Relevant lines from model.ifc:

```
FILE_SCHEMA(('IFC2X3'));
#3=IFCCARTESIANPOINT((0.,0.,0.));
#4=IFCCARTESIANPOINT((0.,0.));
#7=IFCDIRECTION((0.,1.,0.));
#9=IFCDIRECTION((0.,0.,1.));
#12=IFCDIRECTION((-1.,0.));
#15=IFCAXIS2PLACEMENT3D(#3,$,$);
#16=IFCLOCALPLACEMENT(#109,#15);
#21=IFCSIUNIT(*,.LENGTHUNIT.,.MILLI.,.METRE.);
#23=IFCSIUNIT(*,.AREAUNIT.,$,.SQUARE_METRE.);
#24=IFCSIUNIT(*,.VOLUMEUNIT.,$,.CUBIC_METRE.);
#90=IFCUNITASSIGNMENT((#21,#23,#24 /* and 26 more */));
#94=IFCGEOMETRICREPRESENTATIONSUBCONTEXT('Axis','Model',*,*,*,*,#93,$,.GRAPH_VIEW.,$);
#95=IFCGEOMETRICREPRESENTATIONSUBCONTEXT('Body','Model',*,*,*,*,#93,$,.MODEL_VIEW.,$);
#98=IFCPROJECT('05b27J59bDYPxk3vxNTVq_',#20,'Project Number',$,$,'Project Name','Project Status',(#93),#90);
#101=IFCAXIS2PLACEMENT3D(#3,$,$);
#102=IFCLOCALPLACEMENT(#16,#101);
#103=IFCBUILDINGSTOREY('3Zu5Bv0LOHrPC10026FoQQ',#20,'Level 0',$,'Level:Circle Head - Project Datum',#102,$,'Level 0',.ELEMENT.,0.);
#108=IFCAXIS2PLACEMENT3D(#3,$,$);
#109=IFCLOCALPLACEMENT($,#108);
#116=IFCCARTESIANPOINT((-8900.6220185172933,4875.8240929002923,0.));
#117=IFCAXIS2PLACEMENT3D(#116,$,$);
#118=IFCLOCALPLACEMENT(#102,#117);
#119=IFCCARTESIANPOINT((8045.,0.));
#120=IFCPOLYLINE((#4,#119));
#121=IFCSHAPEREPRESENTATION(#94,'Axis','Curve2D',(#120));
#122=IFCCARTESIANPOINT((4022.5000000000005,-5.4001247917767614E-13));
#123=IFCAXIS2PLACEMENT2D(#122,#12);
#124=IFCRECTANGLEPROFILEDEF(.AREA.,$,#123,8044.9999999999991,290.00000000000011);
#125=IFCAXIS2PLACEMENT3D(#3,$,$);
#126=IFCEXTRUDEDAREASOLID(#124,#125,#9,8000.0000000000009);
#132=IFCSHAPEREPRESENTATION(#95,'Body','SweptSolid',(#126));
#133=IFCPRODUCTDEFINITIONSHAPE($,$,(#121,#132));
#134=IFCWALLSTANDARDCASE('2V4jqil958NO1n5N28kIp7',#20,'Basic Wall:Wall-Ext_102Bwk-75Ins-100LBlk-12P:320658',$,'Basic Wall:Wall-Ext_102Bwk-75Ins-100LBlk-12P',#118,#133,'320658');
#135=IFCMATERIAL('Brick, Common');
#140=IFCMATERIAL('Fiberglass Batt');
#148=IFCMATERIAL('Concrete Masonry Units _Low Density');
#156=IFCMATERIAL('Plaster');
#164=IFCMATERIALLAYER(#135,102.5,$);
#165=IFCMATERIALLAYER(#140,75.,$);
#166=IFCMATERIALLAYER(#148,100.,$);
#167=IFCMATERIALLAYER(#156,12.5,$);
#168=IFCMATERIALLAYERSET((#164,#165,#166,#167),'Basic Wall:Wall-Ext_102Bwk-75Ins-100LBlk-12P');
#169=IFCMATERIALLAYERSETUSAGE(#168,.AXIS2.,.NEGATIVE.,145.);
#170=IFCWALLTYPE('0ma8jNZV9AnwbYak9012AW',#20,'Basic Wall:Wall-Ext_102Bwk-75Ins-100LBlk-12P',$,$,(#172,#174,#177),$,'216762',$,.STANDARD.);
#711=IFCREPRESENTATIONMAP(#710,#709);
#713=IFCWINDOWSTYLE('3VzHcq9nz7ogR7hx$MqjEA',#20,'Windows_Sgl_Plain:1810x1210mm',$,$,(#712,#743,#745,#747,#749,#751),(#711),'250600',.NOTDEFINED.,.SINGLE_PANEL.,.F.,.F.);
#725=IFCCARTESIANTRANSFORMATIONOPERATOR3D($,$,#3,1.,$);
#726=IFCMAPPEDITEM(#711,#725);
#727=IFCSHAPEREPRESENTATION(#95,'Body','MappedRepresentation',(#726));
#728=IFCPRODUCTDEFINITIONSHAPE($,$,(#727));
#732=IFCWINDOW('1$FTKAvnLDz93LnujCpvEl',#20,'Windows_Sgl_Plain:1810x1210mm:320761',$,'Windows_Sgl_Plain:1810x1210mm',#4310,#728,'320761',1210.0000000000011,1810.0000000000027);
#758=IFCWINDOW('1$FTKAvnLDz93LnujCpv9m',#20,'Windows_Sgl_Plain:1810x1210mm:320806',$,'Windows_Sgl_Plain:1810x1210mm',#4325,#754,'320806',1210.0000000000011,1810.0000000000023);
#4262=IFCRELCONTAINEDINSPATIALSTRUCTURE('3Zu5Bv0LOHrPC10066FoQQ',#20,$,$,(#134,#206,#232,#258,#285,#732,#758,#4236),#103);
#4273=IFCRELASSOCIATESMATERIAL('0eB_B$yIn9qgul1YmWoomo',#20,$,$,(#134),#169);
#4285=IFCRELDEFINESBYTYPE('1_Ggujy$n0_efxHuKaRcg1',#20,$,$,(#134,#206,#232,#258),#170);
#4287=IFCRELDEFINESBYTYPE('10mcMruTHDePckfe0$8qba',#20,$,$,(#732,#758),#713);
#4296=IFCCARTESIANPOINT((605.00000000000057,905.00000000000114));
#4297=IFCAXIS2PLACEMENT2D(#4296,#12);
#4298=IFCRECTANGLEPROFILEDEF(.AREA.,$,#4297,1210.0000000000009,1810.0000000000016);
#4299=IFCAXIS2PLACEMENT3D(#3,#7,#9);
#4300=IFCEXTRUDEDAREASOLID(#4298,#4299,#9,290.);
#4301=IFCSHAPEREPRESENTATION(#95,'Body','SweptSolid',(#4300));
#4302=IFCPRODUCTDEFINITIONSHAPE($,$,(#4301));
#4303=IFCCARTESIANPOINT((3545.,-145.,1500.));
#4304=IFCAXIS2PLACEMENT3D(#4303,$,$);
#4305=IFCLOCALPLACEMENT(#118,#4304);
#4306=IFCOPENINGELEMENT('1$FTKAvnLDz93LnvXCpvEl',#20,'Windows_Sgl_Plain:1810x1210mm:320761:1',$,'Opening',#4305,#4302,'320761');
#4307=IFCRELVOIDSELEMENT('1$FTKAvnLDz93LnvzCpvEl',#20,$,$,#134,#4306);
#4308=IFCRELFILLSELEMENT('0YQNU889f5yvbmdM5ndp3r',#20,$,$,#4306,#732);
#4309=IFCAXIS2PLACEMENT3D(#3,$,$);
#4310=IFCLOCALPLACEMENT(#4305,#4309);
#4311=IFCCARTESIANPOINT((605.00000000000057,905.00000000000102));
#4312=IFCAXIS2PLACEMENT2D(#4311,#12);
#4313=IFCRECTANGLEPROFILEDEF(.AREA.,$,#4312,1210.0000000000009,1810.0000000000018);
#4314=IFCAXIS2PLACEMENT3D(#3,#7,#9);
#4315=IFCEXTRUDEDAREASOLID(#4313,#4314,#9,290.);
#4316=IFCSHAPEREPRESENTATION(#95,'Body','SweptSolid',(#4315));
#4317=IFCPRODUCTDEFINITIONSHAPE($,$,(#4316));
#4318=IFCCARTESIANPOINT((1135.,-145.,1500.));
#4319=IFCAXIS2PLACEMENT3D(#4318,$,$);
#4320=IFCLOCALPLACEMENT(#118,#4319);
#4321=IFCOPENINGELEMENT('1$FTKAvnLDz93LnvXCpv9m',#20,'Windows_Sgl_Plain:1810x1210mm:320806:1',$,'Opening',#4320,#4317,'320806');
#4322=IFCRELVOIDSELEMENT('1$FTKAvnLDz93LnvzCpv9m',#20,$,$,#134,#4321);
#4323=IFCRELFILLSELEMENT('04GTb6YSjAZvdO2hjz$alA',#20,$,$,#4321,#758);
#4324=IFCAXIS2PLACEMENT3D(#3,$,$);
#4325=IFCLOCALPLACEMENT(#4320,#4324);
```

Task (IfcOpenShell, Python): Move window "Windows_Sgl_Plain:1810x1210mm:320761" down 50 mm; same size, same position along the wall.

```python
import numpy as np
import ifcopenshell
import ifcopenshell.api.geometry
import ifcopenshell.util.placement
import ifcopenshell.util.unit

model = ifcopenshell.open("model.ifc")
unit_scale = ifcopenshell.util.unit.calculate_unit_scale(model)

window = model.by_guid("1$FTKAvnLDz93LnujCpvEl")
opening = window.FillsVoids[0].RelatingOpeningElement
dz = -50.0

shift = np.array([0.0, 0.0, dz])
# The window is placed relative to its opening, so it follows when the opening moves.
matrix = ifcopenshell.util.placement.get_local_placement(opening.ObjectPlacement)
matrix[:3, 3] += shift
ifcopenshell.api.geometry.edit_object_placement(
    model, product=opening, matrix=matrix, is_si=False, should_transform_children=True
)

print(f"moved by {dz * unit_scale:+.3f} m")

model.write("model_updated.ifc")
```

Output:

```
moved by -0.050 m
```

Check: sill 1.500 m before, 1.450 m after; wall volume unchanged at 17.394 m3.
